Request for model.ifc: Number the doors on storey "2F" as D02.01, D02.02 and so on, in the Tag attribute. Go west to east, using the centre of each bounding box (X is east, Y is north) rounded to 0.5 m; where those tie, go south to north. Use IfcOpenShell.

First a look at what the model holds.

```python
import ifcopenshell
import ifcopenshell.util.element
import ifcopenshell.util.placement

model = ifcopenshell.open("model.ifc")
print(model.schema)
storey = next(s for s in model.by_type("IfcBuildingStorey") if s.Name == "2F")
doors = [e for e in ifcopenshell.util.element.get_decomposition(storey) if e.is_a("IfcDoor")]
for e in sorted(doors, key=lambda e: e.id()):
    origin = ifcopenshell.util.placement.get_local_placement(e.ObjectPlacement)[:3, 3]
    print(e.id(), e.Tag, e.Name, origin.round(2) + 0.0, sep=" | ")
```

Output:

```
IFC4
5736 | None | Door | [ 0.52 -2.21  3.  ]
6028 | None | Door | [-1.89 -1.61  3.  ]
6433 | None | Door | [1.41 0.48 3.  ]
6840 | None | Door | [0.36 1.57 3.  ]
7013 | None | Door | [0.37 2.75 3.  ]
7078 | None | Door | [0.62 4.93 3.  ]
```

```python
import ifcopenshell
import ifcopenshell.geom
import ifcopenshell.util.element
import ifcopenshell.util.shape

model = ifcopenshell.open("model.ifc")
settings = ifcopenshell.geom.settings()
settings.set("use-world-coords", True)


def centre(element):
    shape = ifcopenshell.geom.create_shape(settings, element)
    return ifcopenshell.util.shape.get_bbox_centroid(shape.geometry)


storey = next(s for s in model.by_type("IfcBuildingStorey") if s.Name == "2F")
doors = [e for e in ifcopenshell.util.element.get_decomposition(storey) if e.is_a("IfcDoor")]

# Insertion points can sit at a corner or the storey origin, so sort by the geometry (in metres).
centres = {e: centre(e) for e in doors}
doors.sort(key=lambda e: (round(centres[e][0] / 0.5), centres[e][1]))

for i, e in enumerate(doors, start=1):
    number = f"D02.{i:02d}"
    e.Tag = number
    print(e.id(), number)

model.write("model_rev.ifc")
```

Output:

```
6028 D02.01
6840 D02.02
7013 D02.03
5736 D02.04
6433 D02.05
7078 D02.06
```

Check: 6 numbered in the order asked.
